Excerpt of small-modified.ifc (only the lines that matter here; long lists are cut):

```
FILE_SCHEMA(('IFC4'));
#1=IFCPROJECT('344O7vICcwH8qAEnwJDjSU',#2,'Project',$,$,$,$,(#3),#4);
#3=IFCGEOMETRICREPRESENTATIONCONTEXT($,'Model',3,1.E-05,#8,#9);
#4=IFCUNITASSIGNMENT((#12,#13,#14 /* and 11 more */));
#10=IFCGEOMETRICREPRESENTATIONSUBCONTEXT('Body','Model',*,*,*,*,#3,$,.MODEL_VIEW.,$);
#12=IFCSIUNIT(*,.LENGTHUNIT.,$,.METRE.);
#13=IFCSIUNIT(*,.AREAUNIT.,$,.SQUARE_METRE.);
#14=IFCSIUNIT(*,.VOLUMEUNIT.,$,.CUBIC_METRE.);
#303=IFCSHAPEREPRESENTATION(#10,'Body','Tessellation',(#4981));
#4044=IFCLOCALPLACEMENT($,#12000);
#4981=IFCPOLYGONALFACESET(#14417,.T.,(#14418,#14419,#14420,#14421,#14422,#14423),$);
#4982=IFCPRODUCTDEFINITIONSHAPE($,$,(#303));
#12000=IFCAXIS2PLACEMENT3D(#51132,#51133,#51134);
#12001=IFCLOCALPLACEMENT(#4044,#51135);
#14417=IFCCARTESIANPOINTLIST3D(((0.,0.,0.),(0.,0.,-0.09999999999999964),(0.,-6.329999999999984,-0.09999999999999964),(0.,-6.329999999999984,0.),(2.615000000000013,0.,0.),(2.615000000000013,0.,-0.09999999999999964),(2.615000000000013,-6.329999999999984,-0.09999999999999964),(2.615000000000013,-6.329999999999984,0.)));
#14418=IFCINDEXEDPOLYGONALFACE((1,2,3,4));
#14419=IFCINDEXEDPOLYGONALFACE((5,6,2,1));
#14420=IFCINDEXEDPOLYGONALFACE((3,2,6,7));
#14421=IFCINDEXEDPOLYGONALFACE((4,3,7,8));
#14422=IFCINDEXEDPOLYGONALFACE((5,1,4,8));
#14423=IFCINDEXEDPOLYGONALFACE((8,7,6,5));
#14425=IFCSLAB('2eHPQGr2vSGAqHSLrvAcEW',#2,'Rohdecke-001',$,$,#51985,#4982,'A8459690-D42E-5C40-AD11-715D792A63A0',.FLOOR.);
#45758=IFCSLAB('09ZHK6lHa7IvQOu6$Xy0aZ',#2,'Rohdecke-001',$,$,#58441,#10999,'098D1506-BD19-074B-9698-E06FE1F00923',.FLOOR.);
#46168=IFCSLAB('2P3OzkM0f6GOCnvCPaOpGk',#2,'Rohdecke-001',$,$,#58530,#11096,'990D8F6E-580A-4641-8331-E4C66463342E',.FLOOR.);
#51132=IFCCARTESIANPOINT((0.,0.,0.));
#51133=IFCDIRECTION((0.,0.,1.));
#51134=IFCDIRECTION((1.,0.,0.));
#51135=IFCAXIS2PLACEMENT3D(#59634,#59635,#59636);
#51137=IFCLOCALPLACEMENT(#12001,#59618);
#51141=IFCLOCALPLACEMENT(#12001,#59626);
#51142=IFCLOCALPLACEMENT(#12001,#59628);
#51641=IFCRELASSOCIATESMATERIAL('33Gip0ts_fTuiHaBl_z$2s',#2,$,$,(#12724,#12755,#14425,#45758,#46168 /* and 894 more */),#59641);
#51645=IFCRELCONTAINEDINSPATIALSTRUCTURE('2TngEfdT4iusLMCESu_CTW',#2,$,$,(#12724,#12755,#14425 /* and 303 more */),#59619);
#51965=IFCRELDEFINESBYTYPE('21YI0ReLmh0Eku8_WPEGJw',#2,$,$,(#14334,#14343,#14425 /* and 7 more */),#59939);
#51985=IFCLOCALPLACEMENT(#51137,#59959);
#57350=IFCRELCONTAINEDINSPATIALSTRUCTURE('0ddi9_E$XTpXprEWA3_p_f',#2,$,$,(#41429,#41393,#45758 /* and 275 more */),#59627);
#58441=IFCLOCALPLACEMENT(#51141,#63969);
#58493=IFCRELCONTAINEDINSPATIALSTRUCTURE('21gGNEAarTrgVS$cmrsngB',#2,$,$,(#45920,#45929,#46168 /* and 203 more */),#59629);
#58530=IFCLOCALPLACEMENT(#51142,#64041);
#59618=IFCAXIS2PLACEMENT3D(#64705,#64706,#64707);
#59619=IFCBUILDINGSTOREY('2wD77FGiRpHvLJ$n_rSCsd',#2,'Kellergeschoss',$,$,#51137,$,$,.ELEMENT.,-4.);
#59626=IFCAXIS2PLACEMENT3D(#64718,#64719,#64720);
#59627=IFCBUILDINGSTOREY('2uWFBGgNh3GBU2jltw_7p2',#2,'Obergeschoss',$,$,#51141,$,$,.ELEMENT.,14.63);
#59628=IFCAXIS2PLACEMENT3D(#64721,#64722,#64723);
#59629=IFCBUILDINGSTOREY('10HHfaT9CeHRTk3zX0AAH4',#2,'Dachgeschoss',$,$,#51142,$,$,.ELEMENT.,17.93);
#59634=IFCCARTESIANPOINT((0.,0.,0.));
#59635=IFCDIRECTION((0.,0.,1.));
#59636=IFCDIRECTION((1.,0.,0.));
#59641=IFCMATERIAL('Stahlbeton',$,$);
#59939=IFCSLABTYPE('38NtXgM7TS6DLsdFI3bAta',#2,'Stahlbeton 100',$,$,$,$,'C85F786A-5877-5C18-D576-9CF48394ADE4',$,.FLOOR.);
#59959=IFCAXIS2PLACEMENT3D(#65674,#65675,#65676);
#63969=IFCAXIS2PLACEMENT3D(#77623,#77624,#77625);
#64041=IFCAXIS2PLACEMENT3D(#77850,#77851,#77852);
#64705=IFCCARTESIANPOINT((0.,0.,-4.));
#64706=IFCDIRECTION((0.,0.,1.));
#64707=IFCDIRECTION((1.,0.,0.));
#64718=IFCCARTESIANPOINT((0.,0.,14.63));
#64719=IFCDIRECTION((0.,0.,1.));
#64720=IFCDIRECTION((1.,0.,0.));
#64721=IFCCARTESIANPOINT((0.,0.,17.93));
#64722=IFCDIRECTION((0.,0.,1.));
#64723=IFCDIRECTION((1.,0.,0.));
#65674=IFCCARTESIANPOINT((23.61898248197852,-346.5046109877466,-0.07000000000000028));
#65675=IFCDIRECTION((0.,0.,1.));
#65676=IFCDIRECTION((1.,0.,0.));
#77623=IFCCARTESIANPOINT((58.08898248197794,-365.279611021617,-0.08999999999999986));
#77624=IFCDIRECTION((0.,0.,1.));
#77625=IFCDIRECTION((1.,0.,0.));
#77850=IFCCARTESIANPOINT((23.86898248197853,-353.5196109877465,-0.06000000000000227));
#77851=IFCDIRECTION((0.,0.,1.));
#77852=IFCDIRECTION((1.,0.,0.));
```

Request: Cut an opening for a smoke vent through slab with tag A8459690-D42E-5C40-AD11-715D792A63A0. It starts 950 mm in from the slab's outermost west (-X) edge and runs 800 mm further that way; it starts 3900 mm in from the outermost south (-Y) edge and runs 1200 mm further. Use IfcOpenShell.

```python
import numpy as np
import ifcopenshell
import ifcopenshell.api.feature
import ifcopenshell.api.geometry
import ifcopenshell.api.root
import ifcopenshell.geom
import ifcopenshell.util.placement
import ifcopenshell.util.representation
import ifcopenshell.util.shape
import ifcopenshell.util.unit

model = ifcopenshell.open("small-modified.ifc")
unit_scale = ifcopenshell.util.unit.calculate_unit_scale(model)
settings = ifcopenshell.geom.settings()


def volume(element):
    """Net volume in cubic metres, openings subtracted."""
    shape = ifcopenshell.geom.create_shape(settings, element)
    return ifcopenshell.util.shape.get_volume(shape.geometry)


slab = model.by_id(14425)
before = volume(slab)

# Extent in the slab's own axes, in metres. The edges named are its -X and -Y sides.
slab_shape = ifcopenshell.geom.create_shape(settings, slab)
vertices = ifcopenshell.util.shape.get_vertices(slab_shape.geometry)
x_min, y_min, bottom = vertices.min(axis=0)
top = vertices[:, 2].max()

opening = ifcopenshell.api.root.create_entity(model, ifc_class="IfcOpeningElement", name="Smoke vent opening", predefined_type="OPENING")
context = ifcopenshell.util.representation.get_context(model, "Model", "Body", "MODEL_VIEW")
width, depth = 0.8, 1.2
outline = [(0.0, 0.0), (width, 0.0), (width, depth), (0.0, depth), (0.0, 0.0)]
# Overshoot both faces by 50 mm so the cut is clean.
shape = ifcopenshell.api.geometry.add_slab_representation(
    model, context=context, depth=top - bottom + 0.1, polyline=outline
)
ifcopenshell.api.geometry.assign_representation(model, product=opening, representation=shape)

matrix = ifcopenshell.util.placement.get_local_placement(slab.ObjectPlacement)
matrix[:, 3] = matrix @ np.append(np.array([x_min + 0.95, y_min + 3.9, bottom - 0.05]) / unit_scale, 1.0)
ifcopenshell.api.geometry.edit_object_placement(model, product=opening, matrix=matrix, is_si=False)
ifcopenshell.api.feature.add_feature(model, feature=opening, element=slab)

after = volume(slab)

print(f"slab volume {before:.3f} -> {after:.3f} m3")

model.write("small-modified-out.ifc")
```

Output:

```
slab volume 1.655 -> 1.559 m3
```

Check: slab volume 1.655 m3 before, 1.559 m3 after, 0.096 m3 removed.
